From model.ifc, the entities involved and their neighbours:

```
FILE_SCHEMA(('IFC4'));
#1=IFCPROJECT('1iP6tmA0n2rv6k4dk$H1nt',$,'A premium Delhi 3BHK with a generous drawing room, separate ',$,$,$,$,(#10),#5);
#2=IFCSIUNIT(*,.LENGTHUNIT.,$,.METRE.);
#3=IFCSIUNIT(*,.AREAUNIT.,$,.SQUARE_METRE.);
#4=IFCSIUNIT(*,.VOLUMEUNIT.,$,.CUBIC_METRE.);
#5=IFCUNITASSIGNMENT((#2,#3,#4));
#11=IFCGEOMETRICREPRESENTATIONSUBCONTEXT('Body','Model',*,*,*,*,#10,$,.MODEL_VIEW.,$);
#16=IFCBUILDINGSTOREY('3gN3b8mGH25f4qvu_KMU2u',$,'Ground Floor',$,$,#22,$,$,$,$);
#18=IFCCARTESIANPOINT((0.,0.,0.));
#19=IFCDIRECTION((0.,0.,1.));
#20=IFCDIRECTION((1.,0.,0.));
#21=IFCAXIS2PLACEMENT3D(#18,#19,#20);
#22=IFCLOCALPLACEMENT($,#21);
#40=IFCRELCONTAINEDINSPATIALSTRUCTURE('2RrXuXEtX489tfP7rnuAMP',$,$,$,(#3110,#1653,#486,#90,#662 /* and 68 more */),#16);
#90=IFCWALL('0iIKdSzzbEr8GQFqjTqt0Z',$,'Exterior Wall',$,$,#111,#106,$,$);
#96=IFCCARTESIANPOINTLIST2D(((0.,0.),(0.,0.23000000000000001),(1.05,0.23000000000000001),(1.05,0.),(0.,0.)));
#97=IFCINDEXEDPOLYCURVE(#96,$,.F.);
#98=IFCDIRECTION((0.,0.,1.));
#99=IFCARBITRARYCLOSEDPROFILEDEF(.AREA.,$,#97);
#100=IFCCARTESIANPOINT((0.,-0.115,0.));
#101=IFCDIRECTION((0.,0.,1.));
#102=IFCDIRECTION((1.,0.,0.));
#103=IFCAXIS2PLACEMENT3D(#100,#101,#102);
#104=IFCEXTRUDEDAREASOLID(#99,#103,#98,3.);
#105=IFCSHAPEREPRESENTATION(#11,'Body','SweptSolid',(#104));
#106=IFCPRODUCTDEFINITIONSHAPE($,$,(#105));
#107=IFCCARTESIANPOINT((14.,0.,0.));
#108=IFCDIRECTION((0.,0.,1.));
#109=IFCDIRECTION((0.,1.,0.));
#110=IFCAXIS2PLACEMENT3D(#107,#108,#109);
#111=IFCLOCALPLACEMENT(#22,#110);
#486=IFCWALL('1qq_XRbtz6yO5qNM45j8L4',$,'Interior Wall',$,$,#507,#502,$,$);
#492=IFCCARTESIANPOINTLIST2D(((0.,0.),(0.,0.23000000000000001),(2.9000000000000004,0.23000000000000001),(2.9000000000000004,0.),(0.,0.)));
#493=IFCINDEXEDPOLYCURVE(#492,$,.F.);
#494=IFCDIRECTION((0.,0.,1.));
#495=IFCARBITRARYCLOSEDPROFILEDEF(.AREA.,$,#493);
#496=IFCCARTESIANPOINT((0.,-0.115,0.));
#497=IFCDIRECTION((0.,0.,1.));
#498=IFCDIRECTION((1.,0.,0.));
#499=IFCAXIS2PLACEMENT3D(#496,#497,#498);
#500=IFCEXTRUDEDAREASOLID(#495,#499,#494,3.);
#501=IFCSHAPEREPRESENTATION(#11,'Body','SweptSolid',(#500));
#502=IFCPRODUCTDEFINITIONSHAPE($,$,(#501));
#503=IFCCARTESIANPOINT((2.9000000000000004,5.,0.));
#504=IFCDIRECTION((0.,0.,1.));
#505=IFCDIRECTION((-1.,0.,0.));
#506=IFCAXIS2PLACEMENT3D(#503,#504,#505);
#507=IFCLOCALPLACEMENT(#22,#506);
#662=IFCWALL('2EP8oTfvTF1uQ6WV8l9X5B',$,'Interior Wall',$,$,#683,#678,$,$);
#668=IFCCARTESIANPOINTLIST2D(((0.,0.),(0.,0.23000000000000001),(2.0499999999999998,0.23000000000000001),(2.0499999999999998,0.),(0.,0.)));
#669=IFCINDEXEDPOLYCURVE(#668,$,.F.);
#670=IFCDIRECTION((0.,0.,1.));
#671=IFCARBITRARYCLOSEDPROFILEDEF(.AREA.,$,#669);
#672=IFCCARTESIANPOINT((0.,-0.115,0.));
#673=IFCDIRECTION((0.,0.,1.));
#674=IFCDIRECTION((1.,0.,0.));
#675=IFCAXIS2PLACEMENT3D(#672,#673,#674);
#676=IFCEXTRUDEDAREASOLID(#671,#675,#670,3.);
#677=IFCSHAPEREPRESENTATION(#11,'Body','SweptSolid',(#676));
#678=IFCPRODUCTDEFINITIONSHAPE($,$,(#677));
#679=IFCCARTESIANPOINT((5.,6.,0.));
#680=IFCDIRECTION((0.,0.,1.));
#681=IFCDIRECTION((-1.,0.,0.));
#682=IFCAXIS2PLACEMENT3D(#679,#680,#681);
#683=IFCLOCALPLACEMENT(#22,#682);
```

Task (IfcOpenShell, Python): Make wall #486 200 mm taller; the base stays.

```python
import ifcopenshell
import ifcopenshell.geom
import ifcopenshell.util.representation
import ifcopenshell.util.shape
import ifcopenshell.util.unit

model = ifcopenshell.open("model.ifc")
unit_scale = ifcopenshell.util.unit.calculate_unit_scale(model)
settings = ifcopenshell.geom.settings()


def volume(element):
    """Net volume in cubic metres, openings subtracted."""
    shape = ifcopenshell.geom.create_shape(settings, element)
    return ifcopenshell.util.shape.get_volume(shape.geometry)


wall = model.by_guid("1qq_XRbtz6yO5qNM45j8L4")
before = volume(wall)

body = ifcopenshell.util.representation.get_representation(wall, "Model", "Body")
solid = body.Items[0]
old_height = solid.Depth
solid.Depth += 0.2 / unit_scale
after = volume(wall)

print(f"height {old_height:g} -> {solid.Depth:g}, volume {before:.3f} -> {after:.3f} m3")

model.write("model_rev.ifc")
```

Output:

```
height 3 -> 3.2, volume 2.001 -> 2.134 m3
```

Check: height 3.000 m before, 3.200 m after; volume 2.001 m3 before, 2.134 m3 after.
